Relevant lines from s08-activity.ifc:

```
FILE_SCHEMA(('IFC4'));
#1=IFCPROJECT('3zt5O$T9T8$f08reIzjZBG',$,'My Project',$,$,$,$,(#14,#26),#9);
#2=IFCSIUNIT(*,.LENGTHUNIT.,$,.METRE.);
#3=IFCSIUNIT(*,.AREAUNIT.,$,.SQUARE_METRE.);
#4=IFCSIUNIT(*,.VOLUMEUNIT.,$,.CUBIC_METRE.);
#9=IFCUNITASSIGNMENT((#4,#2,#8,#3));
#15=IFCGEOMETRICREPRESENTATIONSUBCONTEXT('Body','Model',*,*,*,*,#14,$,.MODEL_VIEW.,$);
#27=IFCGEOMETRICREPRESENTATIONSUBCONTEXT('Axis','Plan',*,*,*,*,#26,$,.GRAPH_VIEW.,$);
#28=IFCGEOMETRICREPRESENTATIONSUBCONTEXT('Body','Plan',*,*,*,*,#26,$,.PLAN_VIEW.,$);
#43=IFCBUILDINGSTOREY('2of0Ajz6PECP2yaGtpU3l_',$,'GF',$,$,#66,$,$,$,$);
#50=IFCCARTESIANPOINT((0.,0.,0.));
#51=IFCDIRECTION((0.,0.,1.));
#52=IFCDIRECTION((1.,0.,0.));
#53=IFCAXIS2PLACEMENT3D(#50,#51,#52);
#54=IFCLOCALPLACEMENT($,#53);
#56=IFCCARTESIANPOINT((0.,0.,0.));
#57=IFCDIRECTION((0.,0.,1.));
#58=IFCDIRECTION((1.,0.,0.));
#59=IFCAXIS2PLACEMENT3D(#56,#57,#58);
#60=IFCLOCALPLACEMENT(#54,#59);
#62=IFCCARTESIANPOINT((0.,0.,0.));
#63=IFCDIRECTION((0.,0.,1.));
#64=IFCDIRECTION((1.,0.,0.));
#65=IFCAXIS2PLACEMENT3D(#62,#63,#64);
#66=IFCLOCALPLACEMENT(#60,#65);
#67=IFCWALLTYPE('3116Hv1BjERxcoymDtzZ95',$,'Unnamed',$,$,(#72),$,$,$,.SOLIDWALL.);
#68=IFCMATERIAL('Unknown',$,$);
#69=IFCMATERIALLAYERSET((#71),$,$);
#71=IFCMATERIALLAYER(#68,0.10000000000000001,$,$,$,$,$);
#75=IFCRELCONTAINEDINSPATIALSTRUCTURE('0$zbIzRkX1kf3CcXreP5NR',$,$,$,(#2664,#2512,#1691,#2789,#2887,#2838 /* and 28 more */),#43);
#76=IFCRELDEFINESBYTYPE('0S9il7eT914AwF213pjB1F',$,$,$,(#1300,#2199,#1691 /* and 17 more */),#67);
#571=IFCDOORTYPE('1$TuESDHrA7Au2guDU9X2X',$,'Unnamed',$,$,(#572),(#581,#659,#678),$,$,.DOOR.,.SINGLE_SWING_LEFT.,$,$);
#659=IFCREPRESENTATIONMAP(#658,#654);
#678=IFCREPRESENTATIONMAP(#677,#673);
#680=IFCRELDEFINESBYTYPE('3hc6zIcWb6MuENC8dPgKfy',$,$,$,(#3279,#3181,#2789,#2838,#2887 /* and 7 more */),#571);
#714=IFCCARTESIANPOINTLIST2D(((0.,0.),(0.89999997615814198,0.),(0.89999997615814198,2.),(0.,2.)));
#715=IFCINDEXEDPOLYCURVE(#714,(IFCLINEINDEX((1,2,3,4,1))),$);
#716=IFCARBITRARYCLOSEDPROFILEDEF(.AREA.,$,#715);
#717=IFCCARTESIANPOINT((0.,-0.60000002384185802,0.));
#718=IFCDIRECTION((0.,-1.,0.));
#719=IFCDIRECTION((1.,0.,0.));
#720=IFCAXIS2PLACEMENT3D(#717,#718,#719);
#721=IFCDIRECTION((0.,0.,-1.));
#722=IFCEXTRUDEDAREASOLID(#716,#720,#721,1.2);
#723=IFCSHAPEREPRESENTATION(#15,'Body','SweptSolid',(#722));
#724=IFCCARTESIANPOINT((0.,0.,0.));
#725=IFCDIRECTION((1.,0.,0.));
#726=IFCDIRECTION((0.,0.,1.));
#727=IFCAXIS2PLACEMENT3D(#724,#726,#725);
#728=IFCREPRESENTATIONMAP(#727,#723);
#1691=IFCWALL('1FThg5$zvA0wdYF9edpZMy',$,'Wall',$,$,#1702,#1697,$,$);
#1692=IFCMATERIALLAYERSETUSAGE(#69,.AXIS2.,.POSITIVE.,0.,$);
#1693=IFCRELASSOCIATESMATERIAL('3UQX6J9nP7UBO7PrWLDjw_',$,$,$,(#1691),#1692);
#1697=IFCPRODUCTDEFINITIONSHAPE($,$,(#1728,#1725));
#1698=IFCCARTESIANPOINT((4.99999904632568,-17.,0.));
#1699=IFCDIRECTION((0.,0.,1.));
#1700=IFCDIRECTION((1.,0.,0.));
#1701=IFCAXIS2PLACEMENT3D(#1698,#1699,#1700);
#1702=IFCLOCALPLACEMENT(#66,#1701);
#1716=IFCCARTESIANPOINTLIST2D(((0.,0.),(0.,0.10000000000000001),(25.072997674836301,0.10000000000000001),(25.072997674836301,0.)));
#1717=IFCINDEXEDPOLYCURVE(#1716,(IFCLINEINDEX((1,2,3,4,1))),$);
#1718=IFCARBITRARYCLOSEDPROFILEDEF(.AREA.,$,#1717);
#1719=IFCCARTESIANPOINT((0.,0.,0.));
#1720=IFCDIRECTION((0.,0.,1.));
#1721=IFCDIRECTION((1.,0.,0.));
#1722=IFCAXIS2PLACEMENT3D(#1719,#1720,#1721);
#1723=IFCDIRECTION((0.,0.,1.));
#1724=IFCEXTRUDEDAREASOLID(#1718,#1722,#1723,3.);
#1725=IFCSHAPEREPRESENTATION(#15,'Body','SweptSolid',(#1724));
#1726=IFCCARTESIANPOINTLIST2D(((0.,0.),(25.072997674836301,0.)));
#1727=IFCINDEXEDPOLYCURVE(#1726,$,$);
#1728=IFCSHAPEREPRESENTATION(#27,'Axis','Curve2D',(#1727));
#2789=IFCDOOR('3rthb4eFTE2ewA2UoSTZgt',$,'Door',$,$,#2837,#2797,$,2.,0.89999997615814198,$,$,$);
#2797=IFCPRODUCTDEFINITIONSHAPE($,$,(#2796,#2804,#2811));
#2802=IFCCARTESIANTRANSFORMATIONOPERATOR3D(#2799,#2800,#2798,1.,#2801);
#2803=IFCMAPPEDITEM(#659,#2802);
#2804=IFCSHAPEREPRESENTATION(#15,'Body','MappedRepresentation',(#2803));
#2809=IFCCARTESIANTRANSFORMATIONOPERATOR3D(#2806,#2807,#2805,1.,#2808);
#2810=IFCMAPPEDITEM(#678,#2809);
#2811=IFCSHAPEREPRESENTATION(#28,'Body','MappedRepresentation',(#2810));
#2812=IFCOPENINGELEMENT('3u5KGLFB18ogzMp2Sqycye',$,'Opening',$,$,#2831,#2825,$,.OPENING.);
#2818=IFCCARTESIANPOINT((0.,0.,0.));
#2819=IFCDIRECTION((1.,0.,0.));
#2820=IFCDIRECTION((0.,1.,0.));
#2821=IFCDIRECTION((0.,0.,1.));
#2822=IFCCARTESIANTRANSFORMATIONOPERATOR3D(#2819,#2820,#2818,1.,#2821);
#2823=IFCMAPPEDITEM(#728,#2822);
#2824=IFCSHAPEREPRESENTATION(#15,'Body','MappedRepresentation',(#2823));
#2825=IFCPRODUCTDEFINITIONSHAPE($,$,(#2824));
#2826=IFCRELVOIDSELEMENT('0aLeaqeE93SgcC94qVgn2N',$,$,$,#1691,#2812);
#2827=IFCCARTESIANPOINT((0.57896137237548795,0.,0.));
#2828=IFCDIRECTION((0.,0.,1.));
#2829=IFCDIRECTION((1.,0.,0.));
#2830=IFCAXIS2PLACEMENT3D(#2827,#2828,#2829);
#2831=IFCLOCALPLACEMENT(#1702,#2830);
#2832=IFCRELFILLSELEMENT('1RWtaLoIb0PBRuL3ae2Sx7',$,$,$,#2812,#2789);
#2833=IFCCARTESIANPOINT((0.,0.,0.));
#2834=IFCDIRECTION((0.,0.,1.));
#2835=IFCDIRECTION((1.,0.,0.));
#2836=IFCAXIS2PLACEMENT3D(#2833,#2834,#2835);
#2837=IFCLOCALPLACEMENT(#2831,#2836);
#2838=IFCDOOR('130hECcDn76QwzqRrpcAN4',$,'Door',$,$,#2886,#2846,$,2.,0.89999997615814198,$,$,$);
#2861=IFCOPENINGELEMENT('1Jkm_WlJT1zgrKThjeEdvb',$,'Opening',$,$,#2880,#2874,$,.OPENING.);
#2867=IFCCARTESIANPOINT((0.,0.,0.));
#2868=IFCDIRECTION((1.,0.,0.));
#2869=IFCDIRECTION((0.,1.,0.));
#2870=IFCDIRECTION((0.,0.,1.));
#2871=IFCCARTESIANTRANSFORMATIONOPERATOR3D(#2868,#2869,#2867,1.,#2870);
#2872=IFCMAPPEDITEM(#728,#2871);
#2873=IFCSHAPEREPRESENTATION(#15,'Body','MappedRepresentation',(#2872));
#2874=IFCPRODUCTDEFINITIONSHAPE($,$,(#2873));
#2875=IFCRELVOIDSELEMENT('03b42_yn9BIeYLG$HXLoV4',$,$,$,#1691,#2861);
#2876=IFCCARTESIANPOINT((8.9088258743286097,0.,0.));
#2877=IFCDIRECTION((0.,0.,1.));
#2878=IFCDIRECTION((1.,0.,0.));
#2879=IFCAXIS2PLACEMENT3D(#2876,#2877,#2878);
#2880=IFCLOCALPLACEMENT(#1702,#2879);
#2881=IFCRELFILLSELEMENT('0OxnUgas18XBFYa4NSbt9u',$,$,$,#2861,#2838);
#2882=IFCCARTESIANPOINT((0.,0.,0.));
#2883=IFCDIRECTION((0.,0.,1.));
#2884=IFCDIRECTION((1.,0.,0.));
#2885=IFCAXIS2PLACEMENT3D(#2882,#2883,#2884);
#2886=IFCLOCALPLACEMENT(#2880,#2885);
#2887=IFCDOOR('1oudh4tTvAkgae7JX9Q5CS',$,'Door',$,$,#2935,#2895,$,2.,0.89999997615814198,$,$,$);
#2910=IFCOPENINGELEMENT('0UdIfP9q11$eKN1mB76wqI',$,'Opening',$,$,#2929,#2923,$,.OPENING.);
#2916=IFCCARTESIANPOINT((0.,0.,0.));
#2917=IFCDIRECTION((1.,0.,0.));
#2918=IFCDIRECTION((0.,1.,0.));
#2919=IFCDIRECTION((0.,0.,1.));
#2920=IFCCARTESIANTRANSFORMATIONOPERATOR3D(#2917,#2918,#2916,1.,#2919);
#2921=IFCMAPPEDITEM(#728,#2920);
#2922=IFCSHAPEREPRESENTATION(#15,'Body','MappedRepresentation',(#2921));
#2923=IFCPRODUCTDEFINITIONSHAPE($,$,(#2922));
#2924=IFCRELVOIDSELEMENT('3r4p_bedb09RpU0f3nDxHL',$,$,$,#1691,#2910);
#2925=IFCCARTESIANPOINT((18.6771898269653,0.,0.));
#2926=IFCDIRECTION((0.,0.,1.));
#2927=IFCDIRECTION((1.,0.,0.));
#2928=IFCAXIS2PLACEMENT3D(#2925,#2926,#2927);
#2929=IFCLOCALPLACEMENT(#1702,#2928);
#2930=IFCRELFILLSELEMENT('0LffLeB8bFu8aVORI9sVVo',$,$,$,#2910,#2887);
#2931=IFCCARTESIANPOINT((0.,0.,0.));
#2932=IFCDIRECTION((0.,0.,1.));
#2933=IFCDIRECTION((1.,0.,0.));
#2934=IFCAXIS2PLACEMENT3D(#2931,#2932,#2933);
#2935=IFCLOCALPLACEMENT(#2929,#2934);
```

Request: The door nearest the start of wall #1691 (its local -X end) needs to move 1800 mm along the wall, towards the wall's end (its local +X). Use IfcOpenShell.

```python
import ifcopenshell
import ifcopenshell.api.geometry
import ifcopenshell.util.placement

model = ifcopenshell.open("s08-activity.ifc")

door = model.by_guid("3rthb4eFTE2ewA2UoSTZgt")
opening = door.FillsVoids[0].RelatingOpeningElement
wall = opening.VoidsElements[0].RelatingBuildingElement

wall_matrix = ifcopenshell.util.placement.get_local_placement(wall.ObjectPlacement)
shift = wall_matrix[:3, 0] * 1.8
before = ifcopenshell.util.placement.get_local_placement(door.ObjectPlacement)[:3, 3].copy()

# The door is placed relative to its opening, so it follows when the opening moves.
matrix = ifcopenshell.util.placement.get_local_placement(opening.ObjectPlacement)
matrix[:3, 3] += shift
ifcopenshell.api.geometry.edit_object_placement(
    model, product=opening, matrix=matrix, is_si=False, should_transform_children=True
)

after = ifcopenshell.util.placement.get_local_placement(door.ObjectPlacement)[:3, 3]
print("door moved by", (after - before).round(3) + 0.0)

model.write("s08-activity-out.ifc")
```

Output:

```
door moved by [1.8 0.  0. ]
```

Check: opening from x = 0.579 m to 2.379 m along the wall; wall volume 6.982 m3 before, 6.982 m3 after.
